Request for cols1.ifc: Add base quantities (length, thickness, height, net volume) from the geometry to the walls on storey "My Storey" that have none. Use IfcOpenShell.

First a look at what the model holds.

```python
import ifcopenshell
import ifcopenshell.util.element
import ifcopenshell.util.unit

model = ifcopenshell.open("cols1.ifc")
print(model.schema)
for unit_type in ("LENGTHUNIT", "AREAUNIT", "VOLUMEUNIT"):
    print(unit_type, ifcopenshell.util.unit.calculate_unit_scale(model, unit_type))
storey = next(s for s in model.by_type("IfcBuildingStorey") if s.Name == "My Storey")
walls = [e for e in ifcopenshell.util.element.get_decomposition(storey) if e.is_a("IfcWall")]
for e in sorted(walls, key=lambda e: e.id()):
    print(e.id(), e.is_a(), e.Name, list(ifcopenshell.util.element.get_psets(e, qtos_only=True)), sep=" | ")
```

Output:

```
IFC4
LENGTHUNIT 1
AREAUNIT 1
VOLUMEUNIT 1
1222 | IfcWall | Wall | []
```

```python
import ifcopenshell
import ifcopenshell.api.pset
import ifcopenshell.geom
import ifcopenshell.util.element
import ifcopenshell.util.shape
import ifcopenshell.util.unit

model = ifcopenshell.open("cols1.ifc")
unit_scale = ifcopenshell.util.unit.calculate_unit_scale(model)
volume_scale = ifcopenshell.util.unit.calculate_unit_scale(model, "VOLUMEUNIT")
settings = ifcopenshell.geom.settings()

storey = next(s for s in model.by_type("IfcBuildingStorey") if s.Name == "My Storey")
walls = [e for e in ifcopenshell.util.element.get_decomposition(storey) if e.is_a("IfcWall")]

for e in sorted(walls, key=lambda e: e.id()):
    if ifcopenshell.util.element.get_psets(e, qtos_only=True, should_inherit=False):
        continue
    # Geometry comes back in metres, in the element's own axes.
    shape = ifcopenshell.geom.create_shape(settings, e)
    values = {
        "Length": ifcopenshell.util.shape.get_x(shape.geometry) / unit_scale,
        "Width": ifcopenshell.util.shape.get_y(shape.geometry) / unit_scale,
        "Height": ifcopenshell.util.shape.get_z(shape.geometry) / unit_scale,
        "NetVolume": ifcopenshell.util.shape.get_volume(shape.geometry) / volume_scale,
    }
    qto = ifcopenshell.api.pset.add_qto(model, product=e, name="Qto_WallBaseQuantities")
    ifcopenshell.api.pset.edit_qto(model, qto=qto, properties=values)
    print(e.id(), {k: round(v, 3) for k, v in values.items()})

model.write("cols1_edited.ifc")
```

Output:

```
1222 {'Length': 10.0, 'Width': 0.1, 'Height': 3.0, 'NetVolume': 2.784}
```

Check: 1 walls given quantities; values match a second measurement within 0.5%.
